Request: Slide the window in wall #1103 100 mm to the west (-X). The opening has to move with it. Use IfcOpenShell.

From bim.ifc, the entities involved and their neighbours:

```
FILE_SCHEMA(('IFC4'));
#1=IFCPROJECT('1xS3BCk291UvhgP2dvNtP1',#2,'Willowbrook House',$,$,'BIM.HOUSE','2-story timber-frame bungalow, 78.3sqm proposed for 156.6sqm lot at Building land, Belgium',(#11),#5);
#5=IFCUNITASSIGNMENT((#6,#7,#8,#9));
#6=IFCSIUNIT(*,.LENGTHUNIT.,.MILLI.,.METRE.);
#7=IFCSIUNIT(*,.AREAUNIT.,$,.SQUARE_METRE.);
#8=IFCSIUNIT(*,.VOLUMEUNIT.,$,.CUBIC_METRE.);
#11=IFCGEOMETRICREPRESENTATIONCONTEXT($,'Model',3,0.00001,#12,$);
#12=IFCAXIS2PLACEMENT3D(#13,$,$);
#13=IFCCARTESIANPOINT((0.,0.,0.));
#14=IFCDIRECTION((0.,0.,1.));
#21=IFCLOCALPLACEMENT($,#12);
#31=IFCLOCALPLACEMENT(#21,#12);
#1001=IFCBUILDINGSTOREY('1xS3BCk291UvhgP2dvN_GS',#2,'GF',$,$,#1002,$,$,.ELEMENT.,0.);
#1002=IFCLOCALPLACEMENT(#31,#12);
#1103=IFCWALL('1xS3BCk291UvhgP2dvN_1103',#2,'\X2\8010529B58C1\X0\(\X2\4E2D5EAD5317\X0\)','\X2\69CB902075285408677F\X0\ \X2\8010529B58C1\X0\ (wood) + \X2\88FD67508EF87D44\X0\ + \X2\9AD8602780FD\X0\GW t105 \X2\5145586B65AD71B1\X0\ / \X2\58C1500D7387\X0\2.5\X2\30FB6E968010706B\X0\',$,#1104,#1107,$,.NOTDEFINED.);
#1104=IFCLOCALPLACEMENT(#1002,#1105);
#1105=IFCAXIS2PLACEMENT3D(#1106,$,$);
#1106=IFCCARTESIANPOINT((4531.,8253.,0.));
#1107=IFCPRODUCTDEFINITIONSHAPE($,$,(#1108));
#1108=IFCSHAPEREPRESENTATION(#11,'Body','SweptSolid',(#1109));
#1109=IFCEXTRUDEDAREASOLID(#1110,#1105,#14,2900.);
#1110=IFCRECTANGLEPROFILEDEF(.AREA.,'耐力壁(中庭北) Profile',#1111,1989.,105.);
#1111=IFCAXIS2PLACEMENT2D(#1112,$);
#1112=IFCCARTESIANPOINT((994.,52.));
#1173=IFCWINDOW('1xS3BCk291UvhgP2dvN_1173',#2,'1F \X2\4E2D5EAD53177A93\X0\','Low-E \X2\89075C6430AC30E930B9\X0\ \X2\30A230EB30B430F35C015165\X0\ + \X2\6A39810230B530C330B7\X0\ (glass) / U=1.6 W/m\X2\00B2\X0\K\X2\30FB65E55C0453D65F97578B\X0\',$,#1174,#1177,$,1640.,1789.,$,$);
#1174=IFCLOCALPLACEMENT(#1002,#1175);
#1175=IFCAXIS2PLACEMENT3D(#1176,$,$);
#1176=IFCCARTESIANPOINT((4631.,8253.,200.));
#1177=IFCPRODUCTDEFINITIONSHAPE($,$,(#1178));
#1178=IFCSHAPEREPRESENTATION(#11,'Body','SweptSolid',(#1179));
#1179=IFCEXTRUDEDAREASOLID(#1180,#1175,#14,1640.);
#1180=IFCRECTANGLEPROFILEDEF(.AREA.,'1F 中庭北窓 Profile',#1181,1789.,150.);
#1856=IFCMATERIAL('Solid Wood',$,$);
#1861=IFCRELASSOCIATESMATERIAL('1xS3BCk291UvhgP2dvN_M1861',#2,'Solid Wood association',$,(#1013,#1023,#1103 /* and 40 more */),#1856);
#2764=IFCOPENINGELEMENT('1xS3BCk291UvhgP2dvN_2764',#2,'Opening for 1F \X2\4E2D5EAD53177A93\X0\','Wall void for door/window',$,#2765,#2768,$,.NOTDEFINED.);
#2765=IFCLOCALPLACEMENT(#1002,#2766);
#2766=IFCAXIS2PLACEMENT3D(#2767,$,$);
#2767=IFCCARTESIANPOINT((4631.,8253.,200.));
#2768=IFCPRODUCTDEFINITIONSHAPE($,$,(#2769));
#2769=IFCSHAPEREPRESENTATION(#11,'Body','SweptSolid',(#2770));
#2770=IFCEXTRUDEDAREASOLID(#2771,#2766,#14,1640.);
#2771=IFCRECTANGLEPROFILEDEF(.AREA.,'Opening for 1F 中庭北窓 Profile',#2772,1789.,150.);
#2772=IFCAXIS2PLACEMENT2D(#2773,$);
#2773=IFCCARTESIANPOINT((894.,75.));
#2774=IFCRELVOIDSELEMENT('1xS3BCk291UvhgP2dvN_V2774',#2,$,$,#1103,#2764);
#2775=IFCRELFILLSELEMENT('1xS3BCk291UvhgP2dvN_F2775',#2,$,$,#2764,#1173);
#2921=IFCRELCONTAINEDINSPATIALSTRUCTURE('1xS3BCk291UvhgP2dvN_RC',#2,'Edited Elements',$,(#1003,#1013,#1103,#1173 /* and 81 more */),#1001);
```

```python
import ifcopenshell
import ifcopenshell.api.geometry
import ifcopenshell.util.placement
import ifcopenshell.util.unit

model = ifcopenshell.open("bim.ifc")
unit_scale = ifcopenshell.util.unit.calculate_unit_scale(model)

window = model.by_id(1173)
opening = window.FillsVoids[0].RelatingOpeningElement
wall = opening.VoidsElements[0].RelatingBuildingElement

wall_matrix = ifcopenshell.util.placement.get_local_placement(wall.ObjectPlacement)
shift = wall_matrix[:3, 0] * -0.1 / unit_scale
before = ifcopenshell.util.placement.get_local_placement(window.ObjectPlacement)[:3, 3].copy()

# The window is not placed relative to its opening, so move both.
for product in (opening, window):
    matrix = ifcopenshell.util.placement.get_local_placement(product.ObjectPlacement)
    matrix[:3, 3] += shift
    ifcopenshell.api.geometry.edit_object_placement(model, product=product, matrix=matrix, is_si=False)

after = ifcopenshell.util.placement.get_local_placement(window.ObjectPlacement)[:3, 3]
print("window moved by", (after - before).round(3) + 0.0)

model.write("bim_edited.ifc")
```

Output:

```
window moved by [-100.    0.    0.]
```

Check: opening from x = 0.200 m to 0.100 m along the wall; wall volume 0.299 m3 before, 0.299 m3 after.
